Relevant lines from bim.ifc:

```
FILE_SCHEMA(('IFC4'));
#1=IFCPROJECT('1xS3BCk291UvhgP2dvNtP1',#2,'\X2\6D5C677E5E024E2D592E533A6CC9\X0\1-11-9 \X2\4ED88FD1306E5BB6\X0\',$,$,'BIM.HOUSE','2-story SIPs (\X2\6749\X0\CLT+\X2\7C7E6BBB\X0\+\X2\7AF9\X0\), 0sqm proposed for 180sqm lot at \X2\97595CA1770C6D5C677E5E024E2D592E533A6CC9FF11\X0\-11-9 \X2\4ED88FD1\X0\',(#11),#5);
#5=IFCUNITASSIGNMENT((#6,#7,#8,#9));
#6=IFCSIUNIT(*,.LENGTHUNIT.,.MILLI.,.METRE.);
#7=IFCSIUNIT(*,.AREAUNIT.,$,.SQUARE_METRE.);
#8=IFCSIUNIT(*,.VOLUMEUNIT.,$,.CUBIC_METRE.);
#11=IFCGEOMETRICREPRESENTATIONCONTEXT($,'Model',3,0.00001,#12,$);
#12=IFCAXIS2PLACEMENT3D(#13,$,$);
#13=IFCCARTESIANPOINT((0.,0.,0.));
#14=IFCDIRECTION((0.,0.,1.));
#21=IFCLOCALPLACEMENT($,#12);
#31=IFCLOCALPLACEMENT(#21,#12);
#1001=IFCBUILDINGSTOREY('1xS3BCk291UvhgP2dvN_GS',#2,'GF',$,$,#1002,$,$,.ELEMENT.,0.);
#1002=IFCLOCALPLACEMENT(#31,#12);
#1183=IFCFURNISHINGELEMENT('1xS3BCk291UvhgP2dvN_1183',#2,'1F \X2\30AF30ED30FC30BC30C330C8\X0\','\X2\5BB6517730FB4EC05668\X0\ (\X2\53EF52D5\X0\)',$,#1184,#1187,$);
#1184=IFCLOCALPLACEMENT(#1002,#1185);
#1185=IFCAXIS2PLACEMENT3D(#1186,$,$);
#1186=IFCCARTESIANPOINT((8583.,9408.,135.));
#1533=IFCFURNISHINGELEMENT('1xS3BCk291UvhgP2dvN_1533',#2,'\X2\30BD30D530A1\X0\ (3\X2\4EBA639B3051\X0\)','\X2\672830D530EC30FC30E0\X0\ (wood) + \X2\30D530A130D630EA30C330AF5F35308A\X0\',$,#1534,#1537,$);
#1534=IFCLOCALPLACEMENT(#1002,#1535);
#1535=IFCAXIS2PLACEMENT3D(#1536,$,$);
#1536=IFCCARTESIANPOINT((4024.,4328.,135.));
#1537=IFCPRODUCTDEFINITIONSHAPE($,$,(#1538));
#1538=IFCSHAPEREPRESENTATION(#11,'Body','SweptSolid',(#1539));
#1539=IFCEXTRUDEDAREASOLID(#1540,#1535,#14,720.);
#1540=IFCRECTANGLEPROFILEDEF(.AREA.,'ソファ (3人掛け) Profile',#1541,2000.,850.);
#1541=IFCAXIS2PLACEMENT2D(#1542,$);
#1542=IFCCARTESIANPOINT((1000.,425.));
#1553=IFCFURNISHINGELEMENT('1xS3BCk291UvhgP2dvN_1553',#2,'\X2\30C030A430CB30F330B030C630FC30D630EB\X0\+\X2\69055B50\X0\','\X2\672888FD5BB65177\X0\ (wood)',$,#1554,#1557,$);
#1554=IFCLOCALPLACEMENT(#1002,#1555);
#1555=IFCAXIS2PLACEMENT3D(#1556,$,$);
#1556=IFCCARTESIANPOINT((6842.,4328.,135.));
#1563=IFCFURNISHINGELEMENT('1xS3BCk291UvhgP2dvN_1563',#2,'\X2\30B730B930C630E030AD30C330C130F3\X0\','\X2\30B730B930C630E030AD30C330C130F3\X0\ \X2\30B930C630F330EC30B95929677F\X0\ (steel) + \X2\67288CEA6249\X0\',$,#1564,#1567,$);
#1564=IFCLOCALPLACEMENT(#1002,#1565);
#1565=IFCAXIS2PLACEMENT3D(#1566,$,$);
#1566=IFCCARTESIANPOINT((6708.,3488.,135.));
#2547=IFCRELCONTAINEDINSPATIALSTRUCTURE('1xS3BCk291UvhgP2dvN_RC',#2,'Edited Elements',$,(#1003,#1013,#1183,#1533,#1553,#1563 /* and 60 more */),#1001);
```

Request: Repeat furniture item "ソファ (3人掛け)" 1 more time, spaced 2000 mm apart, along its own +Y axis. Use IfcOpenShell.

```python
import ifcopenshell
import ifcopenshell.api.geometry
import ifcopenshell.api.root
import ifcopenshell.util.element
import ifcopenshell.util.placement
import ifcopenshell.util.unit

model = ifcopenshell.open("bim.ifc")
unit_scale = ifcopenshell.util.unit.calculate_unit_scale(model)


def reuse_history(source, copy):
    """copy_class also copies each property set's owner history, people and application; keep the originals."""
    for rel in copy.IsDefinedBy:
        if rel.is_a("IfcRelDefinesByProperties") and (history := rel.RelatingPropertyDefinition.OwnerHistory):
            rel.RelatingPropertyDefinition.OwnerHistory = source.OwnerHistory
            ifcopenshell.util.element.remove_deep2(model, history)


source = model.by_guid("1xS3BCk291UvhgP2dvN_1533")
base = ifcopenshell.util.placement.get_local_placement(source.ObjectPlacement)
step = base[:3, 1] * 2 / unit_scale

for i in range(1, 2):
    copy = ifcopenshell.api.root.copy_class(model, product=source)
    copy.Representation = ifcopenshell.util.element.copy_deep(
        model, source.Representation, exclude=["IfcGeometricRepresentationContext", "IfcRepresentationMap"]
    )
    reuse_history(source, copy)
    matrix = base.copy()
    matrix[:3, 3] += i * step
    print("added at", matrix[:3, 3].round(3) + 0.0)
    ifcopenshell.api.geometry.edit_object_placement(model, product=copy, matrix=matrix, is_si=False)

model.write("bim-out.ifc")
```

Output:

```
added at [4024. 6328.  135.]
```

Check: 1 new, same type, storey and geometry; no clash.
